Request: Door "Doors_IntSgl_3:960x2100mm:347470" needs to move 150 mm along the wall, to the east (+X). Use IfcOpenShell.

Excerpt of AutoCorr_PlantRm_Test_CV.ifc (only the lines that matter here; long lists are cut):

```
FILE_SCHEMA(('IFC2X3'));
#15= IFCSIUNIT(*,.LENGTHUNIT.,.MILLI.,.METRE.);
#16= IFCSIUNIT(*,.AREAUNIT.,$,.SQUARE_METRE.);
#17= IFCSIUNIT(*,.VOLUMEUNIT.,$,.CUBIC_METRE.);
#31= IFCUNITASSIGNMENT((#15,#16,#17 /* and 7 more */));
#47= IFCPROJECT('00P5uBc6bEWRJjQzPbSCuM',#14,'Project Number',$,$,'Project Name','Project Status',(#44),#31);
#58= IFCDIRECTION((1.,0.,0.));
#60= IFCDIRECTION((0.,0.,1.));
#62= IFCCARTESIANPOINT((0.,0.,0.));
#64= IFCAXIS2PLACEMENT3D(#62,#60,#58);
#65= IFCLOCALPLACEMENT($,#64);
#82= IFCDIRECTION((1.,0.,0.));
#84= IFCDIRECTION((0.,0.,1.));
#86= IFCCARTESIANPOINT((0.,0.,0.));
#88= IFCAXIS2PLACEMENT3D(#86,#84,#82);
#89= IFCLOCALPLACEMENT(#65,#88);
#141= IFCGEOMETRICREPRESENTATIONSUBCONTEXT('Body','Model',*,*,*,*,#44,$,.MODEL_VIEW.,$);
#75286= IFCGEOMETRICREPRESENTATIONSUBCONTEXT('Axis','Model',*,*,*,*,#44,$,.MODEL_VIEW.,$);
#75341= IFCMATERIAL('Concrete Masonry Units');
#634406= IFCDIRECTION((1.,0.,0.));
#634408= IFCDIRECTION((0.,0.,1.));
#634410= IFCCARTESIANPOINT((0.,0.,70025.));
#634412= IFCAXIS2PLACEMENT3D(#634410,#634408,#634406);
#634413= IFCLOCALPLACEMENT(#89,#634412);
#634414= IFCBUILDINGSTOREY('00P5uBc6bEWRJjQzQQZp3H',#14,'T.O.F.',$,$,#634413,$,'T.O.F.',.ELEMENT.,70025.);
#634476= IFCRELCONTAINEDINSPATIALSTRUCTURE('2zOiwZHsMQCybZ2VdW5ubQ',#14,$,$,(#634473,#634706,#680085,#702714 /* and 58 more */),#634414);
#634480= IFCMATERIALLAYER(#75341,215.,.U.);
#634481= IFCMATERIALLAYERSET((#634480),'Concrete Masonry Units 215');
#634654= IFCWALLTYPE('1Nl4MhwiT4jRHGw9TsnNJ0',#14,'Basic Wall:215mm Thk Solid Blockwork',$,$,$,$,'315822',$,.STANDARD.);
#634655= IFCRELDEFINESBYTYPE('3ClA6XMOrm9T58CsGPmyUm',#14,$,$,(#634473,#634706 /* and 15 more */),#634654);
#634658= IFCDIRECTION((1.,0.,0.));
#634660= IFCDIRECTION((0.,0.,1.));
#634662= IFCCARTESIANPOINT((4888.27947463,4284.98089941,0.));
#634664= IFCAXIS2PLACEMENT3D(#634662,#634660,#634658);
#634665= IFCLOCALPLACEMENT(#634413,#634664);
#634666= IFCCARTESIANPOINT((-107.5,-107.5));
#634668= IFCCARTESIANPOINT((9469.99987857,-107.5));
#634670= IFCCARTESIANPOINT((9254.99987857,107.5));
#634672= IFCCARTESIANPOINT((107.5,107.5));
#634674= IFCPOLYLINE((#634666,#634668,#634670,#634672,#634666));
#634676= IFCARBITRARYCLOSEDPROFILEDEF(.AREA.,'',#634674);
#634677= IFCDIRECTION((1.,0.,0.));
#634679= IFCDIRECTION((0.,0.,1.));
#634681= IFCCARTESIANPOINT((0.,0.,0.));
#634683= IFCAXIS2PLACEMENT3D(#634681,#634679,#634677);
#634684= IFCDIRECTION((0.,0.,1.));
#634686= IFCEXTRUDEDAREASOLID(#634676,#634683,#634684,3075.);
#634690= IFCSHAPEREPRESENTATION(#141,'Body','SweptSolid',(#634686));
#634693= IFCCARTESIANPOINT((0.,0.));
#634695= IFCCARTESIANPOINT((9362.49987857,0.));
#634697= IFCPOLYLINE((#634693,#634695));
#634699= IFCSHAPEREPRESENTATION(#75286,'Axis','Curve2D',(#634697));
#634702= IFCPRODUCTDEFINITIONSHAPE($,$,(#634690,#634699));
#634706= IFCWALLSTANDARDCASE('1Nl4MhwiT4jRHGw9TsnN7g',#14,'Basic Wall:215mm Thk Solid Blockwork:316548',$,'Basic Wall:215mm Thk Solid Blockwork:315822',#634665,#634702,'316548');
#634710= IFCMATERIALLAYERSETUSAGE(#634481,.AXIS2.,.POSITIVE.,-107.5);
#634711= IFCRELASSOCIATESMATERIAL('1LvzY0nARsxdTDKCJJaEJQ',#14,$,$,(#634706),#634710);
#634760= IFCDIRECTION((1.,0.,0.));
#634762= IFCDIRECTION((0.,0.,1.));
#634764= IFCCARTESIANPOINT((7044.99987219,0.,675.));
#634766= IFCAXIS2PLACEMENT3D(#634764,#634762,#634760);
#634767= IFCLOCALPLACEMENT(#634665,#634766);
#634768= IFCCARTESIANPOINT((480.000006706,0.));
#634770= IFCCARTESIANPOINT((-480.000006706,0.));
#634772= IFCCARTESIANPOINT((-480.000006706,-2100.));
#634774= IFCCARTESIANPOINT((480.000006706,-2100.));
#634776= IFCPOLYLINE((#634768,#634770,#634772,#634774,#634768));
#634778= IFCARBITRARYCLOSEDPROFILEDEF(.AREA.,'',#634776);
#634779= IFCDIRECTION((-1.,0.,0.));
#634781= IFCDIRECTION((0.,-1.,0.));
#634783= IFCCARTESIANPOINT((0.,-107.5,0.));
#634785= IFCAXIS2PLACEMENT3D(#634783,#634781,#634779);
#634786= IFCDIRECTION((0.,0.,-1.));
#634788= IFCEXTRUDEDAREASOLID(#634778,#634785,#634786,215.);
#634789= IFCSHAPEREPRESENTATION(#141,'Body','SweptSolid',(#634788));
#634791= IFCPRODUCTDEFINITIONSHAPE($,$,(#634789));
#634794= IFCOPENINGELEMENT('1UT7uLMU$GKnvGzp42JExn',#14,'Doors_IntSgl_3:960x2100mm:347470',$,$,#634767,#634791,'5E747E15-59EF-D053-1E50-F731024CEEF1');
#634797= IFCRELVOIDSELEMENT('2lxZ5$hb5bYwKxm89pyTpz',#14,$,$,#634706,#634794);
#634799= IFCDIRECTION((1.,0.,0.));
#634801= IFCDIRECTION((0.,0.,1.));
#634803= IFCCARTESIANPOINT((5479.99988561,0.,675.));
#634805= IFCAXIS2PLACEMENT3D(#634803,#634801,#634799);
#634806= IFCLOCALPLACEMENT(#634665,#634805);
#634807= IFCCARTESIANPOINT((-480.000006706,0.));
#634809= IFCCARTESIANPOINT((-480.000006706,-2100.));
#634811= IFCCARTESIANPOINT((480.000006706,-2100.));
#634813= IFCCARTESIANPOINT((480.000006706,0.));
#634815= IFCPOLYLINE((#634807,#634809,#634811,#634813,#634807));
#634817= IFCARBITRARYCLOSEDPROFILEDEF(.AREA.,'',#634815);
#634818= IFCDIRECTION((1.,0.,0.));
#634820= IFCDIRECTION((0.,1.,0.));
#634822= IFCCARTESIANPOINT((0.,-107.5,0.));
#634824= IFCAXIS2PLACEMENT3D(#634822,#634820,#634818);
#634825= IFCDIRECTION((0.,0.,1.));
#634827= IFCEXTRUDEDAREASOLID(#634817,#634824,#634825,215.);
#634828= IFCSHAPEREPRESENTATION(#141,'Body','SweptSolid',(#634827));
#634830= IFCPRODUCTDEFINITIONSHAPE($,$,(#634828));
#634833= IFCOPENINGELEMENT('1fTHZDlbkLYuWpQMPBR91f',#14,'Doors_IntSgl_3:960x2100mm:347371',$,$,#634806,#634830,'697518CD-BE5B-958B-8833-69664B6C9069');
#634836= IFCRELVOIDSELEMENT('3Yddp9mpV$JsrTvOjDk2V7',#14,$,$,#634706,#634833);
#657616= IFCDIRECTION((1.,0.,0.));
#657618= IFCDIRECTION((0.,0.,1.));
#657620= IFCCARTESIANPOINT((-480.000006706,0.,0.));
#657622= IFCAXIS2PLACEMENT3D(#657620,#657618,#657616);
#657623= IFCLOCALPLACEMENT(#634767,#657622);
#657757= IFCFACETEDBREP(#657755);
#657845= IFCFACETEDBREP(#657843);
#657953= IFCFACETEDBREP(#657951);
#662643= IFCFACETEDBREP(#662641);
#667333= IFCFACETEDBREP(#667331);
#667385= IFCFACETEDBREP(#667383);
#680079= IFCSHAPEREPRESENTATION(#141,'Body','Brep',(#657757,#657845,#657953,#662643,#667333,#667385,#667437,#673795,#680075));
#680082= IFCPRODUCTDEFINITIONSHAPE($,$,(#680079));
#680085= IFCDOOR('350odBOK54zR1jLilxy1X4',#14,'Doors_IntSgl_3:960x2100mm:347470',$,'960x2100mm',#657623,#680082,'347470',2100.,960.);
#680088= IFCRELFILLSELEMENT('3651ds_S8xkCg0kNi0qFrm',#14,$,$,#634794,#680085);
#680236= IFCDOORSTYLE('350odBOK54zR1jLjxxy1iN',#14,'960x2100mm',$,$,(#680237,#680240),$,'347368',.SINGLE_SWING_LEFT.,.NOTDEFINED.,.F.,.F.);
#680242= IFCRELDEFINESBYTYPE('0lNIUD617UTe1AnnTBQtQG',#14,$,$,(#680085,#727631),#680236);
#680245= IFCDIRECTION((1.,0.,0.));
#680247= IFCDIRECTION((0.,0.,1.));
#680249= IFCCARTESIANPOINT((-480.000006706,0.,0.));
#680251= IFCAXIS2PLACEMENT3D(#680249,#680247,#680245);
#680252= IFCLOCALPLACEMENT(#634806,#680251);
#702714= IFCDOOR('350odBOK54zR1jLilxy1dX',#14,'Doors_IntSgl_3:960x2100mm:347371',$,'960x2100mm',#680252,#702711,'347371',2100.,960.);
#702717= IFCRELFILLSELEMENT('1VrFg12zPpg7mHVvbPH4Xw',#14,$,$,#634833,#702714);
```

```python
import ifcopenshell
import ifcopenshell.api.geometry
import ifcopenshell.util.placement
import ifcopenshell.util.unit

model = ifcopenshell.open("AutoCorr_PlantRm_Test_CV.ifc")
unit_scale = ifcopenshell.util.unit.calculate_unit_scale(model)

door = model.by_guid("350odBOK54zR1jLilxy1X4")
opening = door.FillsVoids[0].RelatingOpeningElement
wall = opening.VoidsElements[0].RelatingBuildingElement

wall_matrix = ifcopenshell.util.placement.get_local_placement(wall.ObjectPlacement)
shift = wall_matrix[:3, 0] * 0.15 / unit_scale
before = ifcopenshell.util.placement.get_local_placement(door.ObjectPlacement)[:3, 3].copy()

# The door is placed relative to its opening, so it follows when the opening moves.
matrix = ifcopenshell.util.placement.get_local_placement(opening.ObjectPlacement)
matrix[:3, 3] += shift
ifcopenshell.api.geometry.edit_object_placement(
    model, product=opening, matrix=matrix, is_si=False, should_transform_children=True
)

after = ifcopenshell.util.placement.get_local_placement(door.ObjectPlacement)[:3, 3]
print("door moved by", (after - before).round(3) + 0.0)

model.write("AutoCorr_PlantRm_Test_CV_rev.ifc")
```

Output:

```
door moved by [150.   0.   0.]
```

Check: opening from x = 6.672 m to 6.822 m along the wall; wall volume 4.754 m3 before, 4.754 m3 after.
